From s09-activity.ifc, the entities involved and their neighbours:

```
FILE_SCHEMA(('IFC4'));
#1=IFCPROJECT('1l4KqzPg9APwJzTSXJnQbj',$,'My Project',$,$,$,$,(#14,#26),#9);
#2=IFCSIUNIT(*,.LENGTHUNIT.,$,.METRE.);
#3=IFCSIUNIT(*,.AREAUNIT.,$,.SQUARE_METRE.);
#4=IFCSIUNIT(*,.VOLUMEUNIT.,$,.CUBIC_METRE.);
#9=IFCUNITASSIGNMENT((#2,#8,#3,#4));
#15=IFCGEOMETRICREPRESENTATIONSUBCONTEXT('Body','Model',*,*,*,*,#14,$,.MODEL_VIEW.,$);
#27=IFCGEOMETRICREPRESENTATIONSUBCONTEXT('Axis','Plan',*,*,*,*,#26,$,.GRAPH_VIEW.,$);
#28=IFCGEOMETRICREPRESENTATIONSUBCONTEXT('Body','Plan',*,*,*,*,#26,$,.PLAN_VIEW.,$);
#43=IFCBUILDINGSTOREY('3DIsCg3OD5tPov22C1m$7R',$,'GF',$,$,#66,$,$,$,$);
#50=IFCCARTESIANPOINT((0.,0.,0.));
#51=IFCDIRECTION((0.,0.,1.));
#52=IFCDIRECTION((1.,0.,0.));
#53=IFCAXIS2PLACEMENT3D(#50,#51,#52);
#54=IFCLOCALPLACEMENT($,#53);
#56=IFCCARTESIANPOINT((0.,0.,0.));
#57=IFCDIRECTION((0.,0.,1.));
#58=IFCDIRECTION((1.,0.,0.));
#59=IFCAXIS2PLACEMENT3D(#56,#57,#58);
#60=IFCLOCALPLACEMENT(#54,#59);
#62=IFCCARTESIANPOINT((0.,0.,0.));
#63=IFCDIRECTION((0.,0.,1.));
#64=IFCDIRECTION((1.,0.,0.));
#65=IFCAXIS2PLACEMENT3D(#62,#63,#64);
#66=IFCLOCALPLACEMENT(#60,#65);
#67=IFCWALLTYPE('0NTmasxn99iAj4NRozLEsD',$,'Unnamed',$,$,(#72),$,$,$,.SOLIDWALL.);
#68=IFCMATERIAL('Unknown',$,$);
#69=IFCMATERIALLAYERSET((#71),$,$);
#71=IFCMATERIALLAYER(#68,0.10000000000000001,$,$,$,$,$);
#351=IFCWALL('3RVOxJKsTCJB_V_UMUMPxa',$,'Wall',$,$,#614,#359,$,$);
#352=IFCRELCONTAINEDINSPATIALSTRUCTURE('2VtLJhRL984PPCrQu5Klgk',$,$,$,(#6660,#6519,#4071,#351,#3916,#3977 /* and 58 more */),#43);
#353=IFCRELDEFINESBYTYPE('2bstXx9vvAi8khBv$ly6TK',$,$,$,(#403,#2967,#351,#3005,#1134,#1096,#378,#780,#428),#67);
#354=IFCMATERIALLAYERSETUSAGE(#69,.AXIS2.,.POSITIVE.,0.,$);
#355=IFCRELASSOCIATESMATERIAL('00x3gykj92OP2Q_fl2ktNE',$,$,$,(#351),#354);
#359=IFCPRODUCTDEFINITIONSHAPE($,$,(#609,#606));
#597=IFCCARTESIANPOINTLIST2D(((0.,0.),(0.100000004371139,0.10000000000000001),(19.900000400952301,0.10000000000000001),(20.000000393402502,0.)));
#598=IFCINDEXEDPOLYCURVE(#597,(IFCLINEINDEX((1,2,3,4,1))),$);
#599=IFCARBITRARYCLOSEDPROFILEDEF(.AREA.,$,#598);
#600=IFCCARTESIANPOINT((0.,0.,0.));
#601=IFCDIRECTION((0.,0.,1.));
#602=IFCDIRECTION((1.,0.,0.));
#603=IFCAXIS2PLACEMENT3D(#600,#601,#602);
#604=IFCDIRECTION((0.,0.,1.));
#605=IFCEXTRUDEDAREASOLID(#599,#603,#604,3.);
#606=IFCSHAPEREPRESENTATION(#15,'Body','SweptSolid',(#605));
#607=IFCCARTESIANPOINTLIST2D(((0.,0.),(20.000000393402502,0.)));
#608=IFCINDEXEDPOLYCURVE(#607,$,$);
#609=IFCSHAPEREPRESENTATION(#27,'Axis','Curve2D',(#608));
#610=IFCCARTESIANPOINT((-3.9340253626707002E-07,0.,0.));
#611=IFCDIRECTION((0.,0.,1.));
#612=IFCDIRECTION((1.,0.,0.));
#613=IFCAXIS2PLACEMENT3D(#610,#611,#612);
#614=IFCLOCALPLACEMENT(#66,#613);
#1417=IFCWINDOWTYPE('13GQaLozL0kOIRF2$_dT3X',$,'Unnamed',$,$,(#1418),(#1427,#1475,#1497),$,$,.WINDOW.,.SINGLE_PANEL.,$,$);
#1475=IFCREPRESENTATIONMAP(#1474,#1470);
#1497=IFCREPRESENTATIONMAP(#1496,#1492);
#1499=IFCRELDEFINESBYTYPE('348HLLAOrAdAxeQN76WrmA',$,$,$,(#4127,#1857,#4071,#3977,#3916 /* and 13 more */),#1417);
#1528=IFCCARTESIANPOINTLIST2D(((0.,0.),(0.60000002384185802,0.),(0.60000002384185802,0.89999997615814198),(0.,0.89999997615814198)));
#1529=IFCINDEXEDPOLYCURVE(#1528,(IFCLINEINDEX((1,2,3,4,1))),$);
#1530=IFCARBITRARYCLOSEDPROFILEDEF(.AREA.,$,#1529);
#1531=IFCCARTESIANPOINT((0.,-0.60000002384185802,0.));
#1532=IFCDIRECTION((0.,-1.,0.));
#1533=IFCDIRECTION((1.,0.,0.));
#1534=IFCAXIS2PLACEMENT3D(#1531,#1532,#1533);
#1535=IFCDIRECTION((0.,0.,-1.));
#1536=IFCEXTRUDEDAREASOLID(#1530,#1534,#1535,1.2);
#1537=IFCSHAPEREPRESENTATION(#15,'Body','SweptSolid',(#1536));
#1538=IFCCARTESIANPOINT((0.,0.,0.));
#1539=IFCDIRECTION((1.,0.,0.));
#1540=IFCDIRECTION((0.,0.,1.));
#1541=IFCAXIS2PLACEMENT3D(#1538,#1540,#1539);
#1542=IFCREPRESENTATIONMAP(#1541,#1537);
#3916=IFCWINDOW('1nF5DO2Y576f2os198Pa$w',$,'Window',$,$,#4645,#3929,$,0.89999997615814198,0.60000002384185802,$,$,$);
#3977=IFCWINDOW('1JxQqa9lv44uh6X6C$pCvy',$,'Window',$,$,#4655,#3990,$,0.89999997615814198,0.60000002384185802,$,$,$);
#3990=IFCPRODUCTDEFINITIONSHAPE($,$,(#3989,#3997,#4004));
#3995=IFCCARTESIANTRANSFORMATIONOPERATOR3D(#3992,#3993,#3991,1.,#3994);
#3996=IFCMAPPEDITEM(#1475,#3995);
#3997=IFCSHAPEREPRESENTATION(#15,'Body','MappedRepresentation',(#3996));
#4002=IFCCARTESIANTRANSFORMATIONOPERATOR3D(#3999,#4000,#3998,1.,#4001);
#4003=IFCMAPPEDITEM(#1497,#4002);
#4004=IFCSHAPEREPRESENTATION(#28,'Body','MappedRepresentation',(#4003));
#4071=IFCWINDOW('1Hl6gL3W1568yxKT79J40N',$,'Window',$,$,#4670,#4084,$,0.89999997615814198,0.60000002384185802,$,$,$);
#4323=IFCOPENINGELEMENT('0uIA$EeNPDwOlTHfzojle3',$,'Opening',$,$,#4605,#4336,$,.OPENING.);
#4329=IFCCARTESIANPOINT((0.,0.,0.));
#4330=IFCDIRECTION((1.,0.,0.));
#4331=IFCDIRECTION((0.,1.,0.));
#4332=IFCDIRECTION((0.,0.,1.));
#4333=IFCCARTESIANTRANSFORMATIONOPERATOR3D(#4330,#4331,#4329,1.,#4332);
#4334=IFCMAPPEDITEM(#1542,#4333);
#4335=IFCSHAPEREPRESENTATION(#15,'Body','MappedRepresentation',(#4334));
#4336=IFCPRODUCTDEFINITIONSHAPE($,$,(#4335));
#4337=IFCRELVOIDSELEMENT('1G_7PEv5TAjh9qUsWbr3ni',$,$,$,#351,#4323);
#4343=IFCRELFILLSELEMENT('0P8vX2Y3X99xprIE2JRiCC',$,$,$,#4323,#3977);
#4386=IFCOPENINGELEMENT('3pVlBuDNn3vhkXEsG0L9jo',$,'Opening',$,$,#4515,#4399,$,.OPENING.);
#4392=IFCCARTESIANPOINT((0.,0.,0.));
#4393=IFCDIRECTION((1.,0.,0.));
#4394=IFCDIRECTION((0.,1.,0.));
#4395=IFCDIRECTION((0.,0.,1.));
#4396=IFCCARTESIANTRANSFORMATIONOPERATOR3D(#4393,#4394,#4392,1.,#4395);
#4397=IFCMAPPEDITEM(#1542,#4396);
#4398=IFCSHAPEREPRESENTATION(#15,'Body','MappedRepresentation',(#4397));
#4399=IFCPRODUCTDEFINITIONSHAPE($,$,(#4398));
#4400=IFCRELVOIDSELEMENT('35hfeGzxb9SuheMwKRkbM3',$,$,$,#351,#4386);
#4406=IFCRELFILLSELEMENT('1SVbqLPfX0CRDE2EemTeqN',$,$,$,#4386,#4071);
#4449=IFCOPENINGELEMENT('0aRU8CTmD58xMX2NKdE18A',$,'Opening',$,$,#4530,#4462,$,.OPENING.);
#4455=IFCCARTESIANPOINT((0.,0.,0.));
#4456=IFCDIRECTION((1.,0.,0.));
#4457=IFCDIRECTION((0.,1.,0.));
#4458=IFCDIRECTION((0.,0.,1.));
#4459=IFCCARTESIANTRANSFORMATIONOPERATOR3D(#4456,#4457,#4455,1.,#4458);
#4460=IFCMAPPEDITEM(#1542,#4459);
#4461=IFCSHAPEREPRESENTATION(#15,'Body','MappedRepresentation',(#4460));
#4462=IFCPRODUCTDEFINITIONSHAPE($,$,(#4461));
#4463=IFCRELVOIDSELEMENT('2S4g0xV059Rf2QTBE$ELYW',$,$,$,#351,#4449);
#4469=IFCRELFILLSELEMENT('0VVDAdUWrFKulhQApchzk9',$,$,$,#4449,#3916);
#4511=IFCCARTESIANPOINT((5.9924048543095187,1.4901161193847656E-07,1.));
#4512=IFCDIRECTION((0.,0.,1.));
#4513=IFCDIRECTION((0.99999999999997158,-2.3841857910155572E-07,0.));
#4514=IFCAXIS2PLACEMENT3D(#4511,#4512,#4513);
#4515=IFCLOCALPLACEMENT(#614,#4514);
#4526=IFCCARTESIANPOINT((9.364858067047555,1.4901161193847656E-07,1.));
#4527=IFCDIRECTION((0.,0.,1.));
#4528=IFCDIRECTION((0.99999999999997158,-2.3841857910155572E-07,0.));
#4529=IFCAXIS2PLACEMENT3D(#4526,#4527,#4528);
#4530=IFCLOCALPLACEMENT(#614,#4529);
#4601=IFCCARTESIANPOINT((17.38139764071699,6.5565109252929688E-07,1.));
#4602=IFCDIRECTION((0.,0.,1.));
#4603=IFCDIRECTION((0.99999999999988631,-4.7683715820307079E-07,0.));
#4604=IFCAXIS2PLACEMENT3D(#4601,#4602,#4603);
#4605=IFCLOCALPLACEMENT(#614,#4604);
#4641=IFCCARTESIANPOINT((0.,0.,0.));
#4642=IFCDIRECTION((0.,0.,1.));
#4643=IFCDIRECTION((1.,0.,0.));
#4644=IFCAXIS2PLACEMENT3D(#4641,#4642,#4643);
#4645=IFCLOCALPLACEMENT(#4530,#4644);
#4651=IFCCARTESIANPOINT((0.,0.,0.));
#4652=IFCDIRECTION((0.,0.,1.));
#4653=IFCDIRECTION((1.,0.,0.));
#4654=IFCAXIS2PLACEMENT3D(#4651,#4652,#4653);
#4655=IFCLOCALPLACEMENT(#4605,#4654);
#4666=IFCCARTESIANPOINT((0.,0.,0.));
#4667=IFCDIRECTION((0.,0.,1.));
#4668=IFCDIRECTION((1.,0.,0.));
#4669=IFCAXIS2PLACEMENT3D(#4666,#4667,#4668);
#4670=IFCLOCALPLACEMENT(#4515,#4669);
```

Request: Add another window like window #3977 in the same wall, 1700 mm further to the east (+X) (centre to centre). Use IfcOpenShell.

```python
import ifcopenshell
import ifcopenshell.api.feature
import ifcopenshell.api.geometry
import ifcopenshell.api.root
import ifcopenshell.geom
import ifcopenshell.util.element
import ifcopenshell.util.placement
import ifcopenshell.util.shape
import ifcopenshell.util.unit

model = ifcopenshell.open("s09-activity.ifc")
unit_scale = ifcopenshell.util.unit.calculate_unit_scale(model)
settings = ifcopenshell.geom.settings()


def volume(element):
    """Net volume in cubic metres, openings subtracted."""
    shape = ifcopenshell.geom.create_shape(settings, element)
    return ifcopenshell.util.shape.get_volume(shape.geometry)


window = model.by_guid("1JxQqa9lv44uh6X6C$pCvy")
opening = window.FillsVoids[0].RelatingOpeningElement
wall = opening.VoidsElements[0].RelatingBuildingElement
before = volume(wall)
shift = ifcopenshell.util.placement.get_local_placement(wall.ObjectPlacement)[:3, 0] * 1.7 / unit_scale

# copy_class copies the void relationship, type, container and properties, but no geometry.
new_opening = ifcopenshell.api.root.copy_class(model, product=opening)
new_opening.Representation = ifcopenshell.util.element.copy_deep(
    model, opening.Representation, exclude=["IfcGeometricRepresentationContext", "IfcRepresentationMap"]
)
new_window = ifcopenshell.api.root.copy_class(model, product=window)
new_window.Representation = ifcopenshell.util.element.copy_deep(
    model, window.Representation, exclude=["IfcGeometricRepresentationContext", "IfcRepresentationMap"]
)
ifcopenshell.api.feature.add_filling(model, opening=new_opening, element=new_window)

for old, new in ((opening, new_opening), (window, new_window)):
    matrix = ifcopenshell.util.placement.get_local_placement(old.ObjectPlacement)
    matrix[:3, 3] += shift
    ifcopenshell.api.geometry.edit_object_placement(model, product=new, matrix=matrix, is_si=False)

after = volume(wall)

print(f"wall volume {before:.3f} -> {after:.3f} m3")

model.write("s09-activity_edited.ifc")
```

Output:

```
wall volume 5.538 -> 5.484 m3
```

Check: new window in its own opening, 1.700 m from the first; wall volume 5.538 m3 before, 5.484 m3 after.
